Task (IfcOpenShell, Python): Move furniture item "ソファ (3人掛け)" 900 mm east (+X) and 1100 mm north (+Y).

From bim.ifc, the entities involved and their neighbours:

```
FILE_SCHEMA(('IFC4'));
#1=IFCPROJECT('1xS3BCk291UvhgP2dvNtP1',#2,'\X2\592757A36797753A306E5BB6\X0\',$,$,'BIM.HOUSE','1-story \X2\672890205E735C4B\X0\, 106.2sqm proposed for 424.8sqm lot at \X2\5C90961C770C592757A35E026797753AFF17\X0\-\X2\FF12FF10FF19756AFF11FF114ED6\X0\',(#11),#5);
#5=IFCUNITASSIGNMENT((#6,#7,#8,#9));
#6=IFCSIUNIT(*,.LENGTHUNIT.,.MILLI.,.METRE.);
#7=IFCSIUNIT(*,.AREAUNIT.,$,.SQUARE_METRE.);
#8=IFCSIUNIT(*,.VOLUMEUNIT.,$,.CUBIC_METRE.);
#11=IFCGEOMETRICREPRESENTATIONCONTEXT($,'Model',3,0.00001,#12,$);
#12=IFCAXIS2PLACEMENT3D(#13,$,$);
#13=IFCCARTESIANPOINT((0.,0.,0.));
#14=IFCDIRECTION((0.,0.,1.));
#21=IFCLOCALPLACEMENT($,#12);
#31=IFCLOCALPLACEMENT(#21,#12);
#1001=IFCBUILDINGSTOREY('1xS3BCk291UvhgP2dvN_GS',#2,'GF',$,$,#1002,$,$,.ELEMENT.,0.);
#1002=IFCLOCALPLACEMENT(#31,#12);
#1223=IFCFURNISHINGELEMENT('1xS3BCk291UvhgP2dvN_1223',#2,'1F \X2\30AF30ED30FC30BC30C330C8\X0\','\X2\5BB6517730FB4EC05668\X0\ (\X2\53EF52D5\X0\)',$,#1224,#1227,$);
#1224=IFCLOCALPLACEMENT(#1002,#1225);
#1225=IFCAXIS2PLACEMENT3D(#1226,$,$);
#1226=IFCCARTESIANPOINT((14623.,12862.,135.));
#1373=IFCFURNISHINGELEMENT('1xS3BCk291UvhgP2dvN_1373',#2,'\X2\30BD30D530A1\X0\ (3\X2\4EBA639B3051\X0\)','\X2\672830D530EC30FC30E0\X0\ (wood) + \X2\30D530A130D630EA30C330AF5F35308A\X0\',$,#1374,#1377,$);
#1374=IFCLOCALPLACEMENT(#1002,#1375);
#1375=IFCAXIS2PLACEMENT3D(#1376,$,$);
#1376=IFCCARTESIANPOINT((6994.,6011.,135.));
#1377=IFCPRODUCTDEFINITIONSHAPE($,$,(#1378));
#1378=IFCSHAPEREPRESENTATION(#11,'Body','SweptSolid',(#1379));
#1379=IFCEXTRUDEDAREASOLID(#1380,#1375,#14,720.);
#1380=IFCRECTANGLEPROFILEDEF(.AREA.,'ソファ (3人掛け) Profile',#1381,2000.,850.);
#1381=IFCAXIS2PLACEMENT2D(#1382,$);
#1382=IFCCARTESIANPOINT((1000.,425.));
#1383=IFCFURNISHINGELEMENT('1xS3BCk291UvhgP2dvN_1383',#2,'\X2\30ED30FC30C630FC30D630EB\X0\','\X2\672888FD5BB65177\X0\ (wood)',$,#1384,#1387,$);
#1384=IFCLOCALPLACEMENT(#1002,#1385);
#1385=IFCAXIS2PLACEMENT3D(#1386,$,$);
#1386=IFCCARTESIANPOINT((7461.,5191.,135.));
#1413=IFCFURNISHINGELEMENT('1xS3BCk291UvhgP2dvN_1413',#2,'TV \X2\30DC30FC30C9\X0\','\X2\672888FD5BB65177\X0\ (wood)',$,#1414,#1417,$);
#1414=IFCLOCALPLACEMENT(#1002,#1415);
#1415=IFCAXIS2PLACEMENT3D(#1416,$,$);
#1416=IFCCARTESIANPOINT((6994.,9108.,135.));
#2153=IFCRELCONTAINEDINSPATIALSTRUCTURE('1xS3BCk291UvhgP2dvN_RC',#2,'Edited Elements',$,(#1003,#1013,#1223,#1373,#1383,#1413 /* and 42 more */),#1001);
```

```python
import ifcopenshell
import ifcopenshell.api.geometry
import ifcopenshell.util.placement
import ifcopenshell.util.unit

model = ifcopenshell.open("bim.ifc")
unit_scale = ifcopenshell.util.unit.calculate_unit_scale(model)

item = model.by_guid("1xS3BCk291UvhgP2dvN_1373")
matrix = ifcopenshell.util.placement.get_local_placement(item.ObjectPlacement)
matrix[0, 3] += 0.9 / unit_scale
matrix[1, 3] += 1.1 / unit_scale
ifcopenshell.api.geometry.edit_object_placement(model, product=item, matrix=matrix, is_si=False)

print(ifcopenshell.util.placement.get_local_placement(item.ObjectPlacement).round(3) + 0.0)

model.write("bim_v2.ifc")
```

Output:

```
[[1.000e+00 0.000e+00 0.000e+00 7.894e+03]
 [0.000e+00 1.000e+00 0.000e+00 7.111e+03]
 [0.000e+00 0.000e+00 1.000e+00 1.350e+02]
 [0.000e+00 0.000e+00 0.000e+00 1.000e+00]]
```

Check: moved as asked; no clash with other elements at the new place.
